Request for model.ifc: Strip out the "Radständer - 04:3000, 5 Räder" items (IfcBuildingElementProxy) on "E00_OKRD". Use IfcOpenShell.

First a look at what the model holds.

```python
import ifcopenshell
import ifcopenshell.util.element

model = ifcopenshell.open("model.ifc")
print(model.schema)
storey = next(s for s in model.by_type("IfcBuildingStorey") if s.Name == "E00_OKRD")
proxies = [e for e in ifcopenshell.util.element.get_decomposition(storey) if e.is_a("IfcBuildingElementProxy")]
seen = {}
for e in proxies:
    element_type = ifcopenshell.util.element.get_type(e)
    name = element_type.Name if element_type not in (None, e) else None
    seen[name] = seen.get(name, 0) + 1
for name, count in sorted(seen.items(), key=str):
    print(count, "x", name)
```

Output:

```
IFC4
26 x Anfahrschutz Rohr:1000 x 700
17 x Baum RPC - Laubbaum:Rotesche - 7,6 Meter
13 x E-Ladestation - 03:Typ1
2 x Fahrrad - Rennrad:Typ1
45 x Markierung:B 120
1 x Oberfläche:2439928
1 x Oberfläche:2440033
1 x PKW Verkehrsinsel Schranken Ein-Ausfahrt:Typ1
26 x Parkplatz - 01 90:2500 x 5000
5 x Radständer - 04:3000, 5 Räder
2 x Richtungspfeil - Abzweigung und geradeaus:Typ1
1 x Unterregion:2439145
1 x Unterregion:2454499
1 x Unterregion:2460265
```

```python
import ifcopenshell
import ifcopenshell.api.root
import ifcopenshell.util.element

model = ifcopenshell.open("model.ifc")

storey = next(s for s in model.by_type("IfcBuildingStorey") if s.Name == "E00_OKRD")
proxies = [e for e in ifcopenshell.util.element.get_decomposition(storey) if e.is_a("IfcBuildingElementProxy")]
targets = [e for e in proxies if (t := ifcopenshell.util.element.get_type(e)) not in (None, e) and t.Name == "Radständer - 04:3000, 5 Räder"]

for e in targets:
    ifcopenshell.api.root.remove_product(model, product=e)
print(len(targets), "removed")

model.write("model_updated.ifc")
```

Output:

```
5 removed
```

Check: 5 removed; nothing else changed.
